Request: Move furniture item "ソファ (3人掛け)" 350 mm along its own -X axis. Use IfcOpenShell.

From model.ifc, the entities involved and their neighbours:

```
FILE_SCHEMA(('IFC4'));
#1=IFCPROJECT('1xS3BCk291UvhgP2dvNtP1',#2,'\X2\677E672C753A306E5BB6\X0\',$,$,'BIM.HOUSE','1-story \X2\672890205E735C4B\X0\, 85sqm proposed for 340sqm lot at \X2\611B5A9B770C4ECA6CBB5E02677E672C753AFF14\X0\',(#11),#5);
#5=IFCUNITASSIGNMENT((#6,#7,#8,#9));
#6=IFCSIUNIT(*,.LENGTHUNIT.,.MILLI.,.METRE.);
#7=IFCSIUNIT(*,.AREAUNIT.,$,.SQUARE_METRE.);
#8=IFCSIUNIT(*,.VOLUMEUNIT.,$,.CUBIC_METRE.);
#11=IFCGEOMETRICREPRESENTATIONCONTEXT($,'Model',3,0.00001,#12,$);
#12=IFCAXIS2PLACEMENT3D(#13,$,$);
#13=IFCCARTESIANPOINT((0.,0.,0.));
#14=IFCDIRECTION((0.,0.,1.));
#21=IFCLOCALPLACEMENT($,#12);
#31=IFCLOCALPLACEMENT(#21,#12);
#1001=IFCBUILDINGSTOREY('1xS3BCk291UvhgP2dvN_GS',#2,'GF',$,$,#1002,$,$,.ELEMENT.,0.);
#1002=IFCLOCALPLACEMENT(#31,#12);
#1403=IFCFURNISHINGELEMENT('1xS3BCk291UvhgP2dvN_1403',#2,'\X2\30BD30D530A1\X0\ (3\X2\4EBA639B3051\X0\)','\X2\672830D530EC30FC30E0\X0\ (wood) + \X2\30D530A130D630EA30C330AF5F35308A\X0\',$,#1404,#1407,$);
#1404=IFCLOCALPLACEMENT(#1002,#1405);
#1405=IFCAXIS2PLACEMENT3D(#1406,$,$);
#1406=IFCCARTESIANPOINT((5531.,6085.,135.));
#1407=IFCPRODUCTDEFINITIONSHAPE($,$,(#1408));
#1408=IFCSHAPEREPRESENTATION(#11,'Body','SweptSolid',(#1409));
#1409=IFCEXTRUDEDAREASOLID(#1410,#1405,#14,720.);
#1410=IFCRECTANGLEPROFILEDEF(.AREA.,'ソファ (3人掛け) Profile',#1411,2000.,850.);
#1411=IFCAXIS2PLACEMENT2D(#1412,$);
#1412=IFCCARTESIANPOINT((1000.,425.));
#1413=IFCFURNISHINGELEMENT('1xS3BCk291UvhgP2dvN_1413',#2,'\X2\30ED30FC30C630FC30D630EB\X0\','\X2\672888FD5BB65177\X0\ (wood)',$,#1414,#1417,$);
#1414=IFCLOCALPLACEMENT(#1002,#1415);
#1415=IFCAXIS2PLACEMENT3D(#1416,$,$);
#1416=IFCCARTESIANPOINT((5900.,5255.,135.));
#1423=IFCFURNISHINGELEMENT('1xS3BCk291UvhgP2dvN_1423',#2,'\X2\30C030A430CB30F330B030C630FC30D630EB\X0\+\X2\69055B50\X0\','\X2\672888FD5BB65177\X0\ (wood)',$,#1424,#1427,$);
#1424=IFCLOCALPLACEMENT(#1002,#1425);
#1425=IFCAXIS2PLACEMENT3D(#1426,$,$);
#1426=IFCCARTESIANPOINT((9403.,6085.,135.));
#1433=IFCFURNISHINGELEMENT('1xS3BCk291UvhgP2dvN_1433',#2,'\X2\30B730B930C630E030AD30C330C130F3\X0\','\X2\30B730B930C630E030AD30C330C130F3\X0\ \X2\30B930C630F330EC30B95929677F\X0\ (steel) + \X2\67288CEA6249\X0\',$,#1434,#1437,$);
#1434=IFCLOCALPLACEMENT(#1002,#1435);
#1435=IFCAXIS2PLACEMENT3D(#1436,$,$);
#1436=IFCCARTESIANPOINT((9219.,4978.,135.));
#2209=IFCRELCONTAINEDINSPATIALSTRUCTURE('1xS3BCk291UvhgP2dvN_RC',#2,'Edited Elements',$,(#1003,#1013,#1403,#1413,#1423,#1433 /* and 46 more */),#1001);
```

```python
import ifcopenshell
import ifcopenshell.api.geometry
import ifcopenshell.util.placement
import ifcopenshell.util.unit

model = ifcopenshell.open("model.ifc")
unit_scale = ifcopenshell.util.unit.calculate_unit_scale(model)

item = model.by_guid("1xS3BCk291UvhgP2dvN_1403")
matrix = ifcopenshell.util.placement.get_local_placement(item.ObjectPlacement)
matrix[:3, 3] -= matrix[:3, 0] * 0.35 / unit_scale
ifcopenshell.api.geometry.edit_object_placement(model, product=item, matrix=matrix, is_si=False)

print(ifcopenshell.util.placement.get_local_placement(item.ObjectPlacement).round(3) + 0.0)

model.write("model_v2.ifc")
```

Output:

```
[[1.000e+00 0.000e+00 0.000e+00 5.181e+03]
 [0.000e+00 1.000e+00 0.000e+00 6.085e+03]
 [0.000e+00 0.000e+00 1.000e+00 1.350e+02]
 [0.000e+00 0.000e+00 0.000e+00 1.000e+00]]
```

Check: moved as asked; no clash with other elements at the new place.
